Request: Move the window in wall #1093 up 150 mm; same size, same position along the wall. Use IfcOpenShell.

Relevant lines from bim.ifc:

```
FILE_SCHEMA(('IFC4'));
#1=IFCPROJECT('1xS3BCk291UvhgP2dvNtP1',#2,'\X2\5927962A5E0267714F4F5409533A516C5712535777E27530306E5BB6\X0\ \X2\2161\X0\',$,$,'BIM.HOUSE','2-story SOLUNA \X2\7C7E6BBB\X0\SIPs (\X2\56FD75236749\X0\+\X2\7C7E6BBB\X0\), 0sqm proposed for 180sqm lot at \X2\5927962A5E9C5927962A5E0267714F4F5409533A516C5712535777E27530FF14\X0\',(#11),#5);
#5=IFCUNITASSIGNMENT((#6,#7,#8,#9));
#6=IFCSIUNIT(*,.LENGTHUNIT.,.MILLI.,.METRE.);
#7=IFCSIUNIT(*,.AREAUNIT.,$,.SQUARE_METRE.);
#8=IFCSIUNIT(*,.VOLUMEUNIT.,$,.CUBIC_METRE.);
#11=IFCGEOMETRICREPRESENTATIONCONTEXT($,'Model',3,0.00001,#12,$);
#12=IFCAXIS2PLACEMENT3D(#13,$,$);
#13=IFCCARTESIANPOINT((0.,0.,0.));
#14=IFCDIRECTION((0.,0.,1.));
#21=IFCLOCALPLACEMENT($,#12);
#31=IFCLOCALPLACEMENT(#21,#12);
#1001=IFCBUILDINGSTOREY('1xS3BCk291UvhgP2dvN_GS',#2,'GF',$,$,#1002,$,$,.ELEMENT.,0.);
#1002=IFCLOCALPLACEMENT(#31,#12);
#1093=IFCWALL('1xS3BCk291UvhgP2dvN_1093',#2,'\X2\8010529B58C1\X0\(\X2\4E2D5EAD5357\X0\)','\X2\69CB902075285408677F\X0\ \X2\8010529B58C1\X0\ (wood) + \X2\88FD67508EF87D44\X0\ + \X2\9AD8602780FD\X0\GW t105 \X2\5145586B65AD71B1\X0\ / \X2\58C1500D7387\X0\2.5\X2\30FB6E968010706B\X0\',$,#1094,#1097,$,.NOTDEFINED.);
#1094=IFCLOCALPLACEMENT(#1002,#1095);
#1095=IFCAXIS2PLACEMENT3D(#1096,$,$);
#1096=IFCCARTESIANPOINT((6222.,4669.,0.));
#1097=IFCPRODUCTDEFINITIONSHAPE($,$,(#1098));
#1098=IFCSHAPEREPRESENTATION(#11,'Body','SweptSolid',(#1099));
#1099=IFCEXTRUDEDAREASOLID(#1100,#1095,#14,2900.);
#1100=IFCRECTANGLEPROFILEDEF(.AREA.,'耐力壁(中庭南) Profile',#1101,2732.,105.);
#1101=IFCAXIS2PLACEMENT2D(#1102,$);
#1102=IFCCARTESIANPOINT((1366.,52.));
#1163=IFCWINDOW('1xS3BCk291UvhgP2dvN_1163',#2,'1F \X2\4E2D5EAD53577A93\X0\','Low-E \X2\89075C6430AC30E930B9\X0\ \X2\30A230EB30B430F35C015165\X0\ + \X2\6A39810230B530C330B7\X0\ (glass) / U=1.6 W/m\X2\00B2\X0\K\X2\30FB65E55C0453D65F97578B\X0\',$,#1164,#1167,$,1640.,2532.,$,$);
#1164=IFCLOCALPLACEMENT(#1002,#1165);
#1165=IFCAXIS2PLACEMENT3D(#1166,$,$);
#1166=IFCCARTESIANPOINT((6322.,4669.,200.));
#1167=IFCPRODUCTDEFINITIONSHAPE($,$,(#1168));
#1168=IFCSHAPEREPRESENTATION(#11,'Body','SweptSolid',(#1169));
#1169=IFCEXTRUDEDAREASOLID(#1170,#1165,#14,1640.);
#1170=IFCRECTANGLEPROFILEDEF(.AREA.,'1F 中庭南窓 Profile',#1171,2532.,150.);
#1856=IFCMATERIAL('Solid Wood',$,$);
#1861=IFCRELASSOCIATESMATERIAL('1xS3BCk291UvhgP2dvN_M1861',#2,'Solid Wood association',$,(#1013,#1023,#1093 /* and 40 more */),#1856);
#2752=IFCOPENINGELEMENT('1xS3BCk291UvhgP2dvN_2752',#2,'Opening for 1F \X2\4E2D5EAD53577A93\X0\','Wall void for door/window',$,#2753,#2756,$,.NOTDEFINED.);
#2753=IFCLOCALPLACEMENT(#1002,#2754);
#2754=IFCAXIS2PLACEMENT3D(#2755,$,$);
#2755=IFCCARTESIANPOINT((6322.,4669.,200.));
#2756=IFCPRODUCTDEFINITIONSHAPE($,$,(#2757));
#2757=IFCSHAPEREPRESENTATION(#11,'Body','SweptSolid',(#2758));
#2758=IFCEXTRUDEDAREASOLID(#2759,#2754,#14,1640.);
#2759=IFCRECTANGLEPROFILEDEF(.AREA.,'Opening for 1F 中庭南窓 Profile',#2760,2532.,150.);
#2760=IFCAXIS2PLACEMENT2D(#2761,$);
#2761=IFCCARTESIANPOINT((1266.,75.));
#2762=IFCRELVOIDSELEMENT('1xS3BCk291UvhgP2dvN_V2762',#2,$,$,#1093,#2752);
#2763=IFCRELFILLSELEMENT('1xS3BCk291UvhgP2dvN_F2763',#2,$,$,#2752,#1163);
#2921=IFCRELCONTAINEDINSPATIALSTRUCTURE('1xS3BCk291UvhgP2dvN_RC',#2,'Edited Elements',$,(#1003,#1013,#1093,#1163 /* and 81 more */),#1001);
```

```python
import numpy as np
import ifcopenshell
import ifcopenshell.api.geometry
import ifcopenshell.util.placement
import ifcopenshell.util.unit

model = ifcopenshell.open("bim.ifc")
unit_scale = ifcopenshell.util.unit.calculate_unit_scale(model)

window = model.by_guid("1xS3BCk291UvhgP2dvN_1163")
opening = window.FillsVoids[0].RelatingOpeningElement
dz = 0.15 / unit_scale

shift = np.array([0.0, 0.0, dz])
# The window is not placed relative to its opening, so move both.
for product in (opening, window):
    matrix = ifcopenshell.util.placement.get_local_placement(product.ObjectPlacement)
    matrix[:3, 3] += shift
    ifcopenshell.api.geometry.edit_object_placement(model, product=product, matrix=matrix, is_si=False)

print(f"moved by {dz * unit_scale:+.3f} m")

model.write("bim_v2.ifc")
```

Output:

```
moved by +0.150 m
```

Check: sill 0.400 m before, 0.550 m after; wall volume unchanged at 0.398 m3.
